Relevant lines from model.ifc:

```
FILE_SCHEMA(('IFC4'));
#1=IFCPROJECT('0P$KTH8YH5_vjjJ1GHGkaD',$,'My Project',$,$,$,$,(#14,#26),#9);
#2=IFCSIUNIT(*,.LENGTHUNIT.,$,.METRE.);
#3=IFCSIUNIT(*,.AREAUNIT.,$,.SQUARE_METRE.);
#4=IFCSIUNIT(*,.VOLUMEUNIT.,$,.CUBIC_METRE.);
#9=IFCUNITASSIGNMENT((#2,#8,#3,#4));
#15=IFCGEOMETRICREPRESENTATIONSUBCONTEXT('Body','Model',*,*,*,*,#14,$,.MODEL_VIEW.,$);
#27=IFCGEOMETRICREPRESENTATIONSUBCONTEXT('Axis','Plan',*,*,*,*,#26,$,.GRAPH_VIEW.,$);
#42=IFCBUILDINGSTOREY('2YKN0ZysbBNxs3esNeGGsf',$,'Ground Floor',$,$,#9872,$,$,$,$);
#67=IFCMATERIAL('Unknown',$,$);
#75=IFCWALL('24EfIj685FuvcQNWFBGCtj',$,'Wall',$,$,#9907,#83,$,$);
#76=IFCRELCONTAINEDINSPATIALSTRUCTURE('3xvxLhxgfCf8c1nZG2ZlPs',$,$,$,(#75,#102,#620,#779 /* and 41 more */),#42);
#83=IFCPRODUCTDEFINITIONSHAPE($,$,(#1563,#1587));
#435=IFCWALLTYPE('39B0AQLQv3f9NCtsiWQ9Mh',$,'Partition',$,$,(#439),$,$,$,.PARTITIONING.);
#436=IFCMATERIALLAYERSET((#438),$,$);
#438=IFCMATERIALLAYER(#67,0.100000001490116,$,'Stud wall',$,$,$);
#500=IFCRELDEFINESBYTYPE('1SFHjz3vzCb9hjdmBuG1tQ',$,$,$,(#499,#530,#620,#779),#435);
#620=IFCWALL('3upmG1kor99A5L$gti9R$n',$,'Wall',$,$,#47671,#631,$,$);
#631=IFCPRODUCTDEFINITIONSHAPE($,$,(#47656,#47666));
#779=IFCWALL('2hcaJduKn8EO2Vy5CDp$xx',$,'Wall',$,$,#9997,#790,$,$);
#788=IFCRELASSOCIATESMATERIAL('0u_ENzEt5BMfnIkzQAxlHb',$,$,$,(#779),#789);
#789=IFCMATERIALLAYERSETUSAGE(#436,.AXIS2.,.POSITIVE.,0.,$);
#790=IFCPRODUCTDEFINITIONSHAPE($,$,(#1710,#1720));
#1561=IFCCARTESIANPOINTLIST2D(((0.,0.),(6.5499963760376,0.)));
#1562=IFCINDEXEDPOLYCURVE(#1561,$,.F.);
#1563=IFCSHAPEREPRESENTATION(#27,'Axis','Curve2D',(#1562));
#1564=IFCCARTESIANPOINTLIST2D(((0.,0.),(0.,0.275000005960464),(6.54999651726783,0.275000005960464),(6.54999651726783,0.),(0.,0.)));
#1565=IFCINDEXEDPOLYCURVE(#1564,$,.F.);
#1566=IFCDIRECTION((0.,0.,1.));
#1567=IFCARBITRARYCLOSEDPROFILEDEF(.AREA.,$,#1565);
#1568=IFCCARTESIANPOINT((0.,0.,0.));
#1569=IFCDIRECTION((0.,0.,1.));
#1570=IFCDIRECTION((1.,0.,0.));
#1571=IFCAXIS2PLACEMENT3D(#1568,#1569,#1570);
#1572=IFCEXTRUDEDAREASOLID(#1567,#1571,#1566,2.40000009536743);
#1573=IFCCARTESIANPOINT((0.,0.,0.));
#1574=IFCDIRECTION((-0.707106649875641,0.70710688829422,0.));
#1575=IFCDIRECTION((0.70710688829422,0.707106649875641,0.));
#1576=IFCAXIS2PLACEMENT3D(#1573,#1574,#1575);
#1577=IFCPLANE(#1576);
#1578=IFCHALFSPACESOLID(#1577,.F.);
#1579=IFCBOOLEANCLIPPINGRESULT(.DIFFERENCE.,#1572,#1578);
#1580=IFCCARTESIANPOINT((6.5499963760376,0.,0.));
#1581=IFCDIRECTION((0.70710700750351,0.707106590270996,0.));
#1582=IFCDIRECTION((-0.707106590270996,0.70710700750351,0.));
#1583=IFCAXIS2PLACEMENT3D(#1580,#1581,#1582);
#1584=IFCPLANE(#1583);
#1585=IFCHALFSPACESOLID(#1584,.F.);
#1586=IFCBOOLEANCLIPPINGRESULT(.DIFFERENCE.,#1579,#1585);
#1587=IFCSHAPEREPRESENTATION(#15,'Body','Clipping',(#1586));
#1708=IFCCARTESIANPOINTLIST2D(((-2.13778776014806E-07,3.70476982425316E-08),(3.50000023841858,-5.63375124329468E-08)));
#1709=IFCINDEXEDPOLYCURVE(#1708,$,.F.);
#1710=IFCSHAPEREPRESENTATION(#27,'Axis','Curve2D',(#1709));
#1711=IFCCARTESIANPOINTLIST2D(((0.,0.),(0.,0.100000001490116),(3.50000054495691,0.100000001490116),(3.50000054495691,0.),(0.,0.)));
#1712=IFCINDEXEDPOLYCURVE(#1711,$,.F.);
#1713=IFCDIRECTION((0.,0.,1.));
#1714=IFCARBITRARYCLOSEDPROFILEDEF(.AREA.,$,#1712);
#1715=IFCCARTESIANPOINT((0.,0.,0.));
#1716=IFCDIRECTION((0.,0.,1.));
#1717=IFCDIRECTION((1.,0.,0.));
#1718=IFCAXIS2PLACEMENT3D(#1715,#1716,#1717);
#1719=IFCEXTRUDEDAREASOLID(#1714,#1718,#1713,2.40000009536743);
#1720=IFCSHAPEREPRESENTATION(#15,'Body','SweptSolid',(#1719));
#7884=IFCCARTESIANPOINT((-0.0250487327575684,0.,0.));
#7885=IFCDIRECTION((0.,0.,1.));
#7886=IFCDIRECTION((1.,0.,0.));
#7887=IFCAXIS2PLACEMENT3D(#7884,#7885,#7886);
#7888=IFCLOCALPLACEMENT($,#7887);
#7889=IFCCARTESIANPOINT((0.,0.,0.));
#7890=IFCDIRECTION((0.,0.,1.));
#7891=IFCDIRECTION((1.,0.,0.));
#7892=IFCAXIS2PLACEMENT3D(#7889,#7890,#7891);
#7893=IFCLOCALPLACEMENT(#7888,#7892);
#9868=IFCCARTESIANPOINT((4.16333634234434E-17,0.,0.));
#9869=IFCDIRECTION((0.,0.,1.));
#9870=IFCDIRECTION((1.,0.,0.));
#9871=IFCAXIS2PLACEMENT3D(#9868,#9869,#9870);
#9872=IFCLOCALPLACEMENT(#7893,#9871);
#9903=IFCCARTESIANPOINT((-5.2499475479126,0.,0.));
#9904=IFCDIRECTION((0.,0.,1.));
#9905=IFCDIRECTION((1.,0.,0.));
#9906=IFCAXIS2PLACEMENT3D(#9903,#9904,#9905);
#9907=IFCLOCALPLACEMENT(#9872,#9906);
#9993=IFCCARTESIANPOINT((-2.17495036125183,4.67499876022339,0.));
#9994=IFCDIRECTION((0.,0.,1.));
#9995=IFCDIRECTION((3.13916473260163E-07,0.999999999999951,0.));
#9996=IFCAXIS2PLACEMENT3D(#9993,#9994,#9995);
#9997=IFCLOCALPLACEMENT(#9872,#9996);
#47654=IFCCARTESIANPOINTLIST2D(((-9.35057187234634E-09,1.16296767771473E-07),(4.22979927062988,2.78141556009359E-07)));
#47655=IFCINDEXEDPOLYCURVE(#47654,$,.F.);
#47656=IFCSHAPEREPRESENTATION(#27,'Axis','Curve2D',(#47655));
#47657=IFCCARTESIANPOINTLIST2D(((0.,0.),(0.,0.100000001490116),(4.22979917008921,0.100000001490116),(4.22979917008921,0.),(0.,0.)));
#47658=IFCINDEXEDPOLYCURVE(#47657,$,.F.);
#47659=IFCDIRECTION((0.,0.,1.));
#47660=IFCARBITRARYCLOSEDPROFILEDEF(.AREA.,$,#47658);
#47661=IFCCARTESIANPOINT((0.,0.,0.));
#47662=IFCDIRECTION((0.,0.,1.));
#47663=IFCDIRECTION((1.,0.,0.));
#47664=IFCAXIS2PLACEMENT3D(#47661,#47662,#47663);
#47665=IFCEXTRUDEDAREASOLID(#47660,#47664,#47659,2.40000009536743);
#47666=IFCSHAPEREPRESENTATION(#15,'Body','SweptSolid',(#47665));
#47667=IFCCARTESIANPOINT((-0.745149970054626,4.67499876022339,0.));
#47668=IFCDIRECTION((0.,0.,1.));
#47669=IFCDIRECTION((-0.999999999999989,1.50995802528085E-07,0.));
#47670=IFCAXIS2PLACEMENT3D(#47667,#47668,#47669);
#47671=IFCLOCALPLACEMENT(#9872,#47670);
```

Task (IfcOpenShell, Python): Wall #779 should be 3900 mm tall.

```python
import ifcopenshell
import ifcopenshell.geom
import ifcopenshell.util.representation
import ifcopenshell.util.shape
import ifcopenshell.util.unit

model = ifcopenshell.open("model.ifc")
unit_scale = ifcopenshell.util.unit.calculate_unit_scale(model)
settings = ifcopenshell.geom.settings()


def volume(element):
    """Net volume in cubic metres, openings subtracted."""
    shape = ifcopenshell.geom.create_shape(settings, element)
    return ifcopenshell.util.shape.get_volume(shape.geometry)


wall = model.by_guid("2hcaJduKn8EO2Vy5CDp$xx")
before = volume(wall)

body = ifcopenshell.util.representation.get_representation(wall, "Model", "Body")
solid = body.Items[0]
old_height = solid.Depth
solid.Depth = 3.9 / unit_scale
after = volume(wall)

print(f"height {old_height:g} -> {solid.Depth:g}, volume {before:.3f} -> {after:.3f} m3")

model.write("model_updated.ifc")
```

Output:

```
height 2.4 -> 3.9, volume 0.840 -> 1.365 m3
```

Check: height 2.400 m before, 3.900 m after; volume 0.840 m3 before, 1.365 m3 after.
